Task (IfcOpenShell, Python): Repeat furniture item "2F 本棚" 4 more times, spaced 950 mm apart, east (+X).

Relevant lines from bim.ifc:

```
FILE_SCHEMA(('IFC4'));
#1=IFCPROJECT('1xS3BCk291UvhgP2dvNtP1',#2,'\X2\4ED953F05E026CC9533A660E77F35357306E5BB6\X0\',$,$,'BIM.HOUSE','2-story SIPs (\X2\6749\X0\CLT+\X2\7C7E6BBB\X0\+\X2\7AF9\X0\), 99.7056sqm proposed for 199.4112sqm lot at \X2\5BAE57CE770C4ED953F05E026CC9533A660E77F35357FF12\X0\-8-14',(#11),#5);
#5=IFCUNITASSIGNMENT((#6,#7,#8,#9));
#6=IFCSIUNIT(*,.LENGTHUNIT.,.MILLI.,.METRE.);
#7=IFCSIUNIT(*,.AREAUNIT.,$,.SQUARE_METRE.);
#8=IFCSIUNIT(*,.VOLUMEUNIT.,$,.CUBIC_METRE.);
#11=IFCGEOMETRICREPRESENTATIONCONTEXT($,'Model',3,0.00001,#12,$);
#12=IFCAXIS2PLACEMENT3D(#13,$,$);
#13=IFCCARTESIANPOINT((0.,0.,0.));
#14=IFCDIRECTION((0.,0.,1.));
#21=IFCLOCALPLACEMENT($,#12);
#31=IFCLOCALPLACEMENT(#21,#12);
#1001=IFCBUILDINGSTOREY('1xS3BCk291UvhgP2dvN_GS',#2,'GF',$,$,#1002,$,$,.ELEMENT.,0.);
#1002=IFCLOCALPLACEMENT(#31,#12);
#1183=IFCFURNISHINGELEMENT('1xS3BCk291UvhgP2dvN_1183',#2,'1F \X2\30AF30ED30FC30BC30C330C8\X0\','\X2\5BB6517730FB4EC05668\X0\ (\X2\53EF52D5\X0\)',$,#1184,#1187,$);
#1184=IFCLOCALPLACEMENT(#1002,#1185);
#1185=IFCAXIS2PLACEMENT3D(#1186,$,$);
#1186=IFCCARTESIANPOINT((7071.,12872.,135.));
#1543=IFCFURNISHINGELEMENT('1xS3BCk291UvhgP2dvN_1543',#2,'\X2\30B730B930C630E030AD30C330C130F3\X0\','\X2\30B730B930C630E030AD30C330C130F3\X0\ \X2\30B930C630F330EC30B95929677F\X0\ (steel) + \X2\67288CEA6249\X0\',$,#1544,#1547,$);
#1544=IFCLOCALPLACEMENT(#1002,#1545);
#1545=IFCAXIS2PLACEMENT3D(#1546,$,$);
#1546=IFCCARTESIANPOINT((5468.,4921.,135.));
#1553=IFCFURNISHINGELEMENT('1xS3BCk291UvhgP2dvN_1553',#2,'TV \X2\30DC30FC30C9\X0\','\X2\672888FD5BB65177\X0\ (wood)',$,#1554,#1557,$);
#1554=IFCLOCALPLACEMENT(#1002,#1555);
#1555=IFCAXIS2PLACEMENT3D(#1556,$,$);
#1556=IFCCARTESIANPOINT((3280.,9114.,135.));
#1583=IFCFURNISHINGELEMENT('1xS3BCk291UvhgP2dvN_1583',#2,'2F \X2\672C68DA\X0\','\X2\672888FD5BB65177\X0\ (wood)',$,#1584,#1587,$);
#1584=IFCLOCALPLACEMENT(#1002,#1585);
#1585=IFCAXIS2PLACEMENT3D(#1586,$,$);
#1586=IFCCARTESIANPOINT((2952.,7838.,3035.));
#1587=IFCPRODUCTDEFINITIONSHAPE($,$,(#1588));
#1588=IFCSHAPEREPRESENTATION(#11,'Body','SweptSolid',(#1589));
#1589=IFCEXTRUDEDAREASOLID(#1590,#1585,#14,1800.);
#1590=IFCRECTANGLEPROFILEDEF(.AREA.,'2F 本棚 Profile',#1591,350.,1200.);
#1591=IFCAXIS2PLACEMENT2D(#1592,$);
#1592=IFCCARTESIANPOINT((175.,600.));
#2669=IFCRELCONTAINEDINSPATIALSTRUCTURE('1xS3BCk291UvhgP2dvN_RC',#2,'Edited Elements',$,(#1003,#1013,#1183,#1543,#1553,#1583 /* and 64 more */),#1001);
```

```python
import numpy as np
import ifcopenshell
import ifcopenshell.api.geometry
import ifcopenshell.api.root
import ifcopenshell.util.element
import ifcopenshell.util.placement
import ifcopenshell.util.unit

model = ifcopenshell.open("bim.ifc")
unit_scale = ifcopenshell.util.unit.calculate_unit_scale(model)


def reuse_history(source, copy):
    """copy_class also copies each property set's owner history, people and application; keep the originals."""
    for rel in copy.IsDefinedBy:
        if rel.is_a("IfcRelDefinesByProperties") and (history := rel.RelatingPropertyDefinition.OwnerHistory):
            rel.RelatingPropertyDefinition.OwnerHistory = source.OwnerHistory
            ifcopenshell.util.element.remove_deep2(model, history)


source = model.by_guid("1xS3BCk291UvhgP2dvN_1583")
base = ifcopenshell.util.placement.get_local_placement(source.ObjectPlacement)
step = np.array([1.0, 0.0, 0.0]) * 0.95 / unit_scale

for i in range(1, 5):
    copy = ifcopenshell.api.root.copy_class(model, product=source)
    copy.Representation = ifcopenshell.util.element.copy_deep(
        model, source.Representation, exclude=["IfcGeometricRepresentationContext", "IfcRepresentationMap"]
    )
    reuse_history(source, copy)
    matrix = base.copy()
    matrix[:3, 3] += i * step
    print("added at", matrix[:3, 3].round(3) + 0.0)
    ifcopenshell.api.geometry.edit_object_placement(model, product=copy, matrix=matrix, is_si=False)

model.write("bim_rev.ifc")
```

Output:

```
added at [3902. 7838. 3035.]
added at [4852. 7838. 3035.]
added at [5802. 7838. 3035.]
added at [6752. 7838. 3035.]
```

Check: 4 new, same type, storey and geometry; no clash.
